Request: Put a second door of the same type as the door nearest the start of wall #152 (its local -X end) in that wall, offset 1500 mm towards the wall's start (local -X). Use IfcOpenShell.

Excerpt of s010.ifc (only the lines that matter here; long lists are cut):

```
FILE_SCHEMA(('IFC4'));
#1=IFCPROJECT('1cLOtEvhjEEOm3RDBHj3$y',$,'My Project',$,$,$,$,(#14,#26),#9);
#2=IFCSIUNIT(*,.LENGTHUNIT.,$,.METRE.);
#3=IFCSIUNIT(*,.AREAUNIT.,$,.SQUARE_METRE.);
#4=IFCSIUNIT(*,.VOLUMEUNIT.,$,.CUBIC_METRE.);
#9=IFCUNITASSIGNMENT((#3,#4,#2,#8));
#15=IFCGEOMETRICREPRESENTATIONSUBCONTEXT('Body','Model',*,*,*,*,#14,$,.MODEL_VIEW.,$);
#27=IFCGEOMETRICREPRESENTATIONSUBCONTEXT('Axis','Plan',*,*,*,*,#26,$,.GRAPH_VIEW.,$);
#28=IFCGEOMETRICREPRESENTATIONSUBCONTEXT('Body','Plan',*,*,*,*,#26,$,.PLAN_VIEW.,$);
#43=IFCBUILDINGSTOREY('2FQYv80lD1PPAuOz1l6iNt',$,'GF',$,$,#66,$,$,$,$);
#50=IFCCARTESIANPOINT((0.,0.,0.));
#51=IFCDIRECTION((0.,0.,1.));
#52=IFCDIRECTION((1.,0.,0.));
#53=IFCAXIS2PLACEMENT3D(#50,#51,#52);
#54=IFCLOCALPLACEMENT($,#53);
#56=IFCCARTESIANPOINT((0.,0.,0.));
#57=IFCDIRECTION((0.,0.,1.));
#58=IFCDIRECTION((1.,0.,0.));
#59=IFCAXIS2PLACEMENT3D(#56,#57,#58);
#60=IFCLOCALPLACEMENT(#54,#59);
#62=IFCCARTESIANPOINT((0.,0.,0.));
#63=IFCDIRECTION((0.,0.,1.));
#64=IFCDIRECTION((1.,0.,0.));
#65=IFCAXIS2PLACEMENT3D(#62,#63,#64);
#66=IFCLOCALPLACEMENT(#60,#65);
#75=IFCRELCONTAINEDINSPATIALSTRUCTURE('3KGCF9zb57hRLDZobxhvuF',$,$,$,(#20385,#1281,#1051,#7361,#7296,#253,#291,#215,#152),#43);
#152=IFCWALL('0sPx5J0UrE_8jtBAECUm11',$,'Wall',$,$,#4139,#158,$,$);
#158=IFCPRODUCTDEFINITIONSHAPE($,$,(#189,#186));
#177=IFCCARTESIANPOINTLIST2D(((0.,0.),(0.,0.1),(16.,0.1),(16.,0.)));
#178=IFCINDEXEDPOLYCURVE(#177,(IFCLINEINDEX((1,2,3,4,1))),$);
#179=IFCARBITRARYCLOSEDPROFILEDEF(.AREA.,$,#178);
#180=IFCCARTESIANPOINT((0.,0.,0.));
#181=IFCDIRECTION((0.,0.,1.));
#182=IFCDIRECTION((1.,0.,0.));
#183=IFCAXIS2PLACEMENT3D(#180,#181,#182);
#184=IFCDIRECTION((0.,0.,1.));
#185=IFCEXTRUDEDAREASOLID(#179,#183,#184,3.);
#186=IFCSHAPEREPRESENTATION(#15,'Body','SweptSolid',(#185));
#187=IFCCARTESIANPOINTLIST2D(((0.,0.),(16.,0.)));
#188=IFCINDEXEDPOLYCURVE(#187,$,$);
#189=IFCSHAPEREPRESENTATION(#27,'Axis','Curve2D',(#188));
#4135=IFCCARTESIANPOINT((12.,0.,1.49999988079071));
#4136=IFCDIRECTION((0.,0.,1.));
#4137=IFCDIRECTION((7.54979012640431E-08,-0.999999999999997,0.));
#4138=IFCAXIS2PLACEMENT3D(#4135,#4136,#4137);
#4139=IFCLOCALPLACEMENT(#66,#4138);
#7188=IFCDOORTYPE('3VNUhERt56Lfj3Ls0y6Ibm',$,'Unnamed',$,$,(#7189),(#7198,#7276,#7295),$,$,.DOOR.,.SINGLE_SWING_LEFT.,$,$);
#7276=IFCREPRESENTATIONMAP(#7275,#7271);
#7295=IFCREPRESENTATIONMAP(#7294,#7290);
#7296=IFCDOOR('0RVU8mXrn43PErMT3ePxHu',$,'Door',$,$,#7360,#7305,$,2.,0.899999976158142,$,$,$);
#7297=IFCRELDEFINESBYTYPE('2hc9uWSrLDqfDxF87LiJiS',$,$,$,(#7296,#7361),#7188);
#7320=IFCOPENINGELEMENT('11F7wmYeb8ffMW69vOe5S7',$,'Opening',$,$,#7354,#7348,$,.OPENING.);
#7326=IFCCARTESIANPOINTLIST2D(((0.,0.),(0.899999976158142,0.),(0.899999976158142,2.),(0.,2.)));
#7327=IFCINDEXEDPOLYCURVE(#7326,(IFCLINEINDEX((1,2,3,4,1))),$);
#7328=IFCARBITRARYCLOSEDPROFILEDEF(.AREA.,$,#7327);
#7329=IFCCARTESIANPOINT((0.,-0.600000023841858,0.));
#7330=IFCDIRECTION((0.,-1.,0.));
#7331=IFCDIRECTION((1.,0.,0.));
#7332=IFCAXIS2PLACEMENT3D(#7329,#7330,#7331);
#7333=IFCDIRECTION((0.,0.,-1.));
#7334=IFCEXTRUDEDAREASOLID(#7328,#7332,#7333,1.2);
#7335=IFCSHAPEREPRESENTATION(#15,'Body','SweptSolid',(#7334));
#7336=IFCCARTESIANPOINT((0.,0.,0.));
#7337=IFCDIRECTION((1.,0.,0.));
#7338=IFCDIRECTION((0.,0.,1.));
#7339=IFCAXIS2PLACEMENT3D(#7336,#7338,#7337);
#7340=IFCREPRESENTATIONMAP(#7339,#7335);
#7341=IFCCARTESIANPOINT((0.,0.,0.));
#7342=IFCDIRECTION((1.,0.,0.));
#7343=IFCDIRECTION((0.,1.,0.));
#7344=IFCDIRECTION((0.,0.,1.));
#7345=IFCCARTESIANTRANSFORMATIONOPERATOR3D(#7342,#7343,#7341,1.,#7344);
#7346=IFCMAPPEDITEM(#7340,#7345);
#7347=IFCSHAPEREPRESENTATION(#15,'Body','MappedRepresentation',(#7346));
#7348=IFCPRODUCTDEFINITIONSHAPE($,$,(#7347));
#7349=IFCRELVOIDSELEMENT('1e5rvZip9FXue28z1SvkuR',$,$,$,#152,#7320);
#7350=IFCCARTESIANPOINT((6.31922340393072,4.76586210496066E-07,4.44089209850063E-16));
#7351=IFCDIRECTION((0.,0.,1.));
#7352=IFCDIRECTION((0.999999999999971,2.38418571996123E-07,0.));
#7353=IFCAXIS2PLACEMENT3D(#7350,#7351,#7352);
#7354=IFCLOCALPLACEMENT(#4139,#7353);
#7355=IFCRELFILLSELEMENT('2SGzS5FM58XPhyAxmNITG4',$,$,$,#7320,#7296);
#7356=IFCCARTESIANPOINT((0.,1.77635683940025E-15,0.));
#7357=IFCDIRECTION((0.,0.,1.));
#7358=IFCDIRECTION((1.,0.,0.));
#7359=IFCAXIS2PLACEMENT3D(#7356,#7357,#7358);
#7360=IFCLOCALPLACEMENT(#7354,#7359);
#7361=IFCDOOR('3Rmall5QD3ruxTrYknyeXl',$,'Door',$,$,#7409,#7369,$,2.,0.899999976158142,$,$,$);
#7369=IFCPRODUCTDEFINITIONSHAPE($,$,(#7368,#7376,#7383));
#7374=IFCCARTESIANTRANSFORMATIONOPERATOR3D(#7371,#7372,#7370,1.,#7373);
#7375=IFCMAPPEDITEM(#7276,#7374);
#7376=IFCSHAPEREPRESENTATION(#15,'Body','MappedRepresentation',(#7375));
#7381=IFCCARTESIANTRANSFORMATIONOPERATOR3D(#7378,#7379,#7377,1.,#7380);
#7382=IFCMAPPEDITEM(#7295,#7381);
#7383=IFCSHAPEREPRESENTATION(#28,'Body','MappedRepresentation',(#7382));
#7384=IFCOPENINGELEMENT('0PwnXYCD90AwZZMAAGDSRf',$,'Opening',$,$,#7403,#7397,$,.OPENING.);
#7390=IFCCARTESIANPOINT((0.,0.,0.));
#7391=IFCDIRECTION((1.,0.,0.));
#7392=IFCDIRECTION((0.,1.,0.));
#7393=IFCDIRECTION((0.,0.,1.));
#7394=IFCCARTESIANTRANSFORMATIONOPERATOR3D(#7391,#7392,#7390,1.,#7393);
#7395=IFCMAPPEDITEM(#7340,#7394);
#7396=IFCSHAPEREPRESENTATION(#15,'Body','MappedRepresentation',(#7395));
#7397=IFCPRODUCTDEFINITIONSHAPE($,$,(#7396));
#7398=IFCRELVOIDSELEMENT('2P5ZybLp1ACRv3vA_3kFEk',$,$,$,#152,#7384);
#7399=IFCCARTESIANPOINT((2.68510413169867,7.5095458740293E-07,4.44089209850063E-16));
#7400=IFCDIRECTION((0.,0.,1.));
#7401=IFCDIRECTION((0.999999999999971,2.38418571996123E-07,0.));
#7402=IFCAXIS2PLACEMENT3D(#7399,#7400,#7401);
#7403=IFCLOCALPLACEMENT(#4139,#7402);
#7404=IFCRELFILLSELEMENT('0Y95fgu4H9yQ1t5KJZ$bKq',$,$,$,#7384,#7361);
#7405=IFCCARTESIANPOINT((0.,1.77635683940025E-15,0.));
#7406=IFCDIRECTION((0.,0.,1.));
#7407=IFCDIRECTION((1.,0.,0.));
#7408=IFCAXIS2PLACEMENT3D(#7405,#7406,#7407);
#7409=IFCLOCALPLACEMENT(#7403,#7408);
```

```python
import ifcopenshell
import ifcopenshell.api.feature
import ifcopenshell.api.geometry
import ifcopenshell.api.root
import ifcopenshell.geom
import ifcopenshell.util.element
import ifcopenshell.util.placement
import ifcopenshell.util.shape
import ifcopenshell.util.unit

model = ifcopenshell.open("s010.ifc")
unit_scale = ifcopenshell.util.unit.calculate_unit_scale(model)
settings = ifcopenshell.geom.settings()


def volume(element):
    """Net volume in cubic metres, openings subtracted."""
    shape = ifcopenshell.geom.create_shape(settings, element)
    return ifcopenshell.util.shape.get_volume(shape.geometry)


door = model.by_guid("3Rmall5QD3ruxTrYknyeXl")
opening = door.FillsVoids[0].RelatingOpeningElement
wall = opening.VoidsElements[0].RelatingBuildingElement
before = volume(wall)
shift = ifcopenshell.util.placement.get_local_placement(wall.ObjectPlacement)[:3, 0] * -1.5 / unit_scale

# copy_class copies the void relationship, type, container and properties, but no geometry.
new_opening = ifcopenshell.api.root.copy_class(model, product=opening)
new_opening.Representation = ifcopenshell.util.element.copy_deep(
    model, opening.Representation, exclude=["IfcGeometricRepresentationContext", "IfcRepresentationMap"]
)
new_door = ifcopenshell.api.root.copy_class(model, product=door)
new_door.Representation = ifcopenshell.util.element.copy_deep(
    model, door.Representation, exclude=["IfcGeometricRepresentationContext", "IfcRepresentationMap"]
)
ifcopenshell.api.feature.add_filling(model, opening=new_opening, element=new_door)

for old, new in ((opening, new_opening), (door, new_door)):
    matrix = ifcopenshell.util.placement.get_local_placement(old.ObjectPlacement)
    matrix[:3, 3] += shift
    ifcopenshell.api.geometry.edit_object_placement(model, product=new, matrix=matrix, is_si=False)

after = volume(wall)

print(f"wall volume {before:.3f} -> {after:.3f} m3")

model.write("s010_rev.ifc")
```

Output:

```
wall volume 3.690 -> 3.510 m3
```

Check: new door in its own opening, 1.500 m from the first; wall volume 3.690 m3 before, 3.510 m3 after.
